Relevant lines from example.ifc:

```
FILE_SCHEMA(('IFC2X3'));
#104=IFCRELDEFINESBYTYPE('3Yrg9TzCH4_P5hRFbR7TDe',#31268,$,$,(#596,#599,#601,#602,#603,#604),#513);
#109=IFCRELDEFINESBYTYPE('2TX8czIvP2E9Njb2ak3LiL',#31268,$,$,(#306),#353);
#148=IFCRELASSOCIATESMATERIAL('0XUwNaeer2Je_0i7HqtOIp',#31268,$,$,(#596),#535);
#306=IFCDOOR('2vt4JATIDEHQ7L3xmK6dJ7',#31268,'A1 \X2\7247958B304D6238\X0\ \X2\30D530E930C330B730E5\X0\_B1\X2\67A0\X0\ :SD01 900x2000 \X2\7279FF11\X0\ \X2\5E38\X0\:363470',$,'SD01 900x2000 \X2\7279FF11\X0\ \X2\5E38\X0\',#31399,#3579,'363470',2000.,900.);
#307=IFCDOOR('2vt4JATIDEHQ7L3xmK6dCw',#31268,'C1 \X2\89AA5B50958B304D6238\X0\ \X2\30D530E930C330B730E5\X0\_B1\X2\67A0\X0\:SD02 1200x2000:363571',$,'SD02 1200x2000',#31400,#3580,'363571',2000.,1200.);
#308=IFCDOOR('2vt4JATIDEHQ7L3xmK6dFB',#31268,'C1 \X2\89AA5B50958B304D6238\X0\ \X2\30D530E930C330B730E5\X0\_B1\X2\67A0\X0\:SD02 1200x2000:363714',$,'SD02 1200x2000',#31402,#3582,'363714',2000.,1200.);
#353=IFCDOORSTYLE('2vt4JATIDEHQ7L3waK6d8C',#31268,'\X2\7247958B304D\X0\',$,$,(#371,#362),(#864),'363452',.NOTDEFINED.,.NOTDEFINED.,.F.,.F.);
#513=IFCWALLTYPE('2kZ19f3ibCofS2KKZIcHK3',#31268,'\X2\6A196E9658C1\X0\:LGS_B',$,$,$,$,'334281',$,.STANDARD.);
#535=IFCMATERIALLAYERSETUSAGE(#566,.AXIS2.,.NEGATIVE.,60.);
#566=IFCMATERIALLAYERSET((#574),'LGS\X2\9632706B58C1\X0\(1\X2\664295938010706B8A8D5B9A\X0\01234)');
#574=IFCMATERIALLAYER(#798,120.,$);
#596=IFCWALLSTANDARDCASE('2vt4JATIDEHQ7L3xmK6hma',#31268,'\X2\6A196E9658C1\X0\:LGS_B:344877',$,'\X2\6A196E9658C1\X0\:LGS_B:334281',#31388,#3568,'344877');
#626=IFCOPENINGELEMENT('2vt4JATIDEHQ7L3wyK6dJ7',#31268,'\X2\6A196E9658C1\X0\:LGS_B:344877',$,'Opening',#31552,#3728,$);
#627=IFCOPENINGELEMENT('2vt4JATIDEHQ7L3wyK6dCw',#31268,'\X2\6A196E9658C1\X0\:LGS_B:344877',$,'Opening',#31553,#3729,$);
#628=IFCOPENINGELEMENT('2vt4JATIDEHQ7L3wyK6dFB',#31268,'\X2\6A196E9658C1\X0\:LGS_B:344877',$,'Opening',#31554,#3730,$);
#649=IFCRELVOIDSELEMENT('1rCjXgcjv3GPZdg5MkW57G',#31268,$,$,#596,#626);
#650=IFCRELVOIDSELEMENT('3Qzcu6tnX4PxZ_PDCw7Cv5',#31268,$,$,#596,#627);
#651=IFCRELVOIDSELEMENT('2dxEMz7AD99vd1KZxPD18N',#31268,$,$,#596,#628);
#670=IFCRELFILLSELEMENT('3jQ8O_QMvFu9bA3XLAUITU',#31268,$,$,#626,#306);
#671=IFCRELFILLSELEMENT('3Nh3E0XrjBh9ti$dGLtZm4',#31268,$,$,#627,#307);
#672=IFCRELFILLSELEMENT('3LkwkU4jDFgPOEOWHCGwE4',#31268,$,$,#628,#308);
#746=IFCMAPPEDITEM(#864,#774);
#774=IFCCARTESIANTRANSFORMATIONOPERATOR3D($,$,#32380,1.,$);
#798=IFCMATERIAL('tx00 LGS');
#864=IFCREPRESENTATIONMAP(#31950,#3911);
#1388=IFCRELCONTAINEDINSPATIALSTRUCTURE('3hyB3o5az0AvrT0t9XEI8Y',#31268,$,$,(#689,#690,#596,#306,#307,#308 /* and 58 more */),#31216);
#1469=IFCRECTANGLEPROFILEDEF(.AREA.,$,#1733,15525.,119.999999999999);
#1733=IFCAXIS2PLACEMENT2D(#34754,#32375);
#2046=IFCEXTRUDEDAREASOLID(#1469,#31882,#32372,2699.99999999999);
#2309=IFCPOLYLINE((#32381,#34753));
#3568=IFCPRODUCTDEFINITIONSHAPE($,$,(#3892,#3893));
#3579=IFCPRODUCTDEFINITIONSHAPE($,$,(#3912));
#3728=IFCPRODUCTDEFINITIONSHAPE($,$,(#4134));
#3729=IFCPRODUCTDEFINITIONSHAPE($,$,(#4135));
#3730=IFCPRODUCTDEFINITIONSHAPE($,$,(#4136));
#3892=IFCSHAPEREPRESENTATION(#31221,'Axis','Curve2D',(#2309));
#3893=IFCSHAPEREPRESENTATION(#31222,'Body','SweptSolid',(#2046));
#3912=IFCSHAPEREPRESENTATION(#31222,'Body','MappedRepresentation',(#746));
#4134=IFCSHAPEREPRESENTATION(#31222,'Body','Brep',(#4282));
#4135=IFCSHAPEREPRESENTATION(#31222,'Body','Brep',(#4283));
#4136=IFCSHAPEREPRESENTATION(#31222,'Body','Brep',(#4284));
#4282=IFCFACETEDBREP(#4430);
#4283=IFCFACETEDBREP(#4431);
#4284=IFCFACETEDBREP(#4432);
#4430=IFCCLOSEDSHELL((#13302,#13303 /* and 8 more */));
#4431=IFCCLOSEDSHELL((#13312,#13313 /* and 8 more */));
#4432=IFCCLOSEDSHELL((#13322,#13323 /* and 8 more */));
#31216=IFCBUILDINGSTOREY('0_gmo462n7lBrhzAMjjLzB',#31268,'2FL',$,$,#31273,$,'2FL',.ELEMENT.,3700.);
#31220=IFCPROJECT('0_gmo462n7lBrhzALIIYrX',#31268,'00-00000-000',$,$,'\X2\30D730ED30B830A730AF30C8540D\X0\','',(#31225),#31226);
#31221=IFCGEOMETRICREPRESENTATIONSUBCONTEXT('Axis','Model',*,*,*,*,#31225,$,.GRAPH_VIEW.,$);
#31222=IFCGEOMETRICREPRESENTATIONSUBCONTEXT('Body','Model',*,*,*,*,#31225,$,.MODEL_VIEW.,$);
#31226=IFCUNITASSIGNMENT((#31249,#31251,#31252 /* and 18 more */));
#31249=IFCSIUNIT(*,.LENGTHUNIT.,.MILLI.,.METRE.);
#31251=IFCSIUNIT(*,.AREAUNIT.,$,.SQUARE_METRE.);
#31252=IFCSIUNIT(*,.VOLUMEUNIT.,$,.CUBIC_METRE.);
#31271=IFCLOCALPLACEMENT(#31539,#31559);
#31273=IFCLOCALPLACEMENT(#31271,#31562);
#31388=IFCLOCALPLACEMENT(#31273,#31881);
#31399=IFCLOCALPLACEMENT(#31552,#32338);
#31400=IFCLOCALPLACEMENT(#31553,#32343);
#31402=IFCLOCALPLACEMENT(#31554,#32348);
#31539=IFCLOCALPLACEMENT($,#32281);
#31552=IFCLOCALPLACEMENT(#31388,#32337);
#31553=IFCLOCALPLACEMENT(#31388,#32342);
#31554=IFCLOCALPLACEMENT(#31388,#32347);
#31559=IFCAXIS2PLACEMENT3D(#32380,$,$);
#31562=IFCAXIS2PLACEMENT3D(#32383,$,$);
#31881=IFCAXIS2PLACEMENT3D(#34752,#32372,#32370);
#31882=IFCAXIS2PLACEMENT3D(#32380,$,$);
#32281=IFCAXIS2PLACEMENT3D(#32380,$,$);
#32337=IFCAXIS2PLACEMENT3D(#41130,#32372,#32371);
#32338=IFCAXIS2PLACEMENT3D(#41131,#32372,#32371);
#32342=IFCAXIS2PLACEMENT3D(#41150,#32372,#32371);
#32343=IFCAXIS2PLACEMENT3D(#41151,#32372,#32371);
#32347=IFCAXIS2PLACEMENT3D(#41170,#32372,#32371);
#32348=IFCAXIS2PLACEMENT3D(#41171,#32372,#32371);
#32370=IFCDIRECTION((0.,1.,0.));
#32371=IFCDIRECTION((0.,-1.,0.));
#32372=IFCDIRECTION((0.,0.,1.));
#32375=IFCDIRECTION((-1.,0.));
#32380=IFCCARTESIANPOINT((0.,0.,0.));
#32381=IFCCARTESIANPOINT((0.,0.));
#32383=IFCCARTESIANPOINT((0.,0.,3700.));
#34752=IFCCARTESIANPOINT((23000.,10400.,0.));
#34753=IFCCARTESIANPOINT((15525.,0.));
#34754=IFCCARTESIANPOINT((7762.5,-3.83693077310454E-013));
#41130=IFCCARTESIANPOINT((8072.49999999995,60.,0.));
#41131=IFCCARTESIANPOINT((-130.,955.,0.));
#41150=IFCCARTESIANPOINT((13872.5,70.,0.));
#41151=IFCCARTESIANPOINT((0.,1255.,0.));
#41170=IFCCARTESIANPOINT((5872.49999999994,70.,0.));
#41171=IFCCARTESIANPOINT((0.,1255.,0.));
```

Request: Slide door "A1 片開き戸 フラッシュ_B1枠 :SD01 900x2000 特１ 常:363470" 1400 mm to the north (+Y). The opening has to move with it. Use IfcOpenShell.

```python
import ifcopenshell
import ifcopenshell.api.geometry
import ifcopenshell.util.placement
import ifcopenshell.util.unit

model = ifcopenshell.open("example.ifc")
unit_scale = ifcopenshell.util.unit.calculate_unit_scale(model)

door = model.by_id(306)
opening = door.FillsVoids[0].RelatingOpeningElement
wall = opening.VoidsElements[0].RelatingBuildingElement

wall_matrix = ifcopenshell.util.placement.get_local_placement(wall.ObjectPlacement)
shift = wall_matrix[:3, 0] * 1.4 / unit_scale
before = ifcopenshell.util.placement.get_local_placement(door.ObjectPlacement)[:3, 3].copy()

# The door is placed relative to its opening, so it follows when the opening moves.
matrix = ifcopenshell.util.placement.get_local_placement(opening.ObjectPlacement)
matrix[:3, 3] += shift
ifcopenshell.api.geometry.edit_object_placement(
    model, product=opening, matrix=matrix, is_si=False, should_transform_children=True
)

after = ifcopenshell.util.placement.get_local_placement(door.ObjectPlacement)[:3, 3]
print("door moved by", (after - before).round(3) + 0.0)

model.write("example_rev.ifc")
```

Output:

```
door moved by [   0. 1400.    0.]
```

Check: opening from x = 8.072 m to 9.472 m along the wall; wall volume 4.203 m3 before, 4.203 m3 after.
